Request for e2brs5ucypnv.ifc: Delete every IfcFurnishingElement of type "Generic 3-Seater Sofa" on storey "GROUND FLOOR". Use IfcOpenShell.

First a look at what the model holds.

```python
import ifcopenshell
import ifcopenshell.util.element

model = ifcopenshell.open("e2brs5ucypnv.ifc")
print(model.schema)
storey = next(s for s in model.by_type("IfcBuildingStorey") if s.Name == "GROUND FLOOR")
furniture = [e for e in ifcopenshell.util.element.get_decomposition(storey) if e.is_a("IfcFurnishingElement")]
seen = {}
for e in furniture:
    element_type = ifcopenshell.util.element.get_type(e)
    name = element_type.Name if element_type not in (None, e) else None
    seen[name] = seen.get(name, 0) + 1
for name, count in sorted(seen.items(), key=str):
    print(count, "x", name)
```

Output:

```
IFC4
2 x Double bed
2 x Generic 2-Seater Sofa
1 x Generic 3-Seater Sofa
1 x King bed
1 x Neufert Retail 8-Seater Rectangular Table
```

```python
import ifcopenshell
import ifcopenshell.api.root
import ifcopenshell.util.element

model = ifcopenshell.open("e2brs5ucypnv.ifc")

storey = next(s for s in model.by_type("IfcBuildingStorey") if s.Name == "GROUND FLOOR")
furniture = [e for e in ifcopenshell.util.element.get_decomposition(storey) if e.is_a("IfcFurnishingElement")]
targets = [e for e in furniture if (t := ifcopenshell.util.element.get_type(e)) not in (None, e) and t.Name == "Generic 3-Seater Sofa"]

for e in targets:
    ifcopenshell.api.root.remove_product(model, product=e)
print(len(targets), "removed")

model.write("e2brs5ucypnv-out.ifc")
```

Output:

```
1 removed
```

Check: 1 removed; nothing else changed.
